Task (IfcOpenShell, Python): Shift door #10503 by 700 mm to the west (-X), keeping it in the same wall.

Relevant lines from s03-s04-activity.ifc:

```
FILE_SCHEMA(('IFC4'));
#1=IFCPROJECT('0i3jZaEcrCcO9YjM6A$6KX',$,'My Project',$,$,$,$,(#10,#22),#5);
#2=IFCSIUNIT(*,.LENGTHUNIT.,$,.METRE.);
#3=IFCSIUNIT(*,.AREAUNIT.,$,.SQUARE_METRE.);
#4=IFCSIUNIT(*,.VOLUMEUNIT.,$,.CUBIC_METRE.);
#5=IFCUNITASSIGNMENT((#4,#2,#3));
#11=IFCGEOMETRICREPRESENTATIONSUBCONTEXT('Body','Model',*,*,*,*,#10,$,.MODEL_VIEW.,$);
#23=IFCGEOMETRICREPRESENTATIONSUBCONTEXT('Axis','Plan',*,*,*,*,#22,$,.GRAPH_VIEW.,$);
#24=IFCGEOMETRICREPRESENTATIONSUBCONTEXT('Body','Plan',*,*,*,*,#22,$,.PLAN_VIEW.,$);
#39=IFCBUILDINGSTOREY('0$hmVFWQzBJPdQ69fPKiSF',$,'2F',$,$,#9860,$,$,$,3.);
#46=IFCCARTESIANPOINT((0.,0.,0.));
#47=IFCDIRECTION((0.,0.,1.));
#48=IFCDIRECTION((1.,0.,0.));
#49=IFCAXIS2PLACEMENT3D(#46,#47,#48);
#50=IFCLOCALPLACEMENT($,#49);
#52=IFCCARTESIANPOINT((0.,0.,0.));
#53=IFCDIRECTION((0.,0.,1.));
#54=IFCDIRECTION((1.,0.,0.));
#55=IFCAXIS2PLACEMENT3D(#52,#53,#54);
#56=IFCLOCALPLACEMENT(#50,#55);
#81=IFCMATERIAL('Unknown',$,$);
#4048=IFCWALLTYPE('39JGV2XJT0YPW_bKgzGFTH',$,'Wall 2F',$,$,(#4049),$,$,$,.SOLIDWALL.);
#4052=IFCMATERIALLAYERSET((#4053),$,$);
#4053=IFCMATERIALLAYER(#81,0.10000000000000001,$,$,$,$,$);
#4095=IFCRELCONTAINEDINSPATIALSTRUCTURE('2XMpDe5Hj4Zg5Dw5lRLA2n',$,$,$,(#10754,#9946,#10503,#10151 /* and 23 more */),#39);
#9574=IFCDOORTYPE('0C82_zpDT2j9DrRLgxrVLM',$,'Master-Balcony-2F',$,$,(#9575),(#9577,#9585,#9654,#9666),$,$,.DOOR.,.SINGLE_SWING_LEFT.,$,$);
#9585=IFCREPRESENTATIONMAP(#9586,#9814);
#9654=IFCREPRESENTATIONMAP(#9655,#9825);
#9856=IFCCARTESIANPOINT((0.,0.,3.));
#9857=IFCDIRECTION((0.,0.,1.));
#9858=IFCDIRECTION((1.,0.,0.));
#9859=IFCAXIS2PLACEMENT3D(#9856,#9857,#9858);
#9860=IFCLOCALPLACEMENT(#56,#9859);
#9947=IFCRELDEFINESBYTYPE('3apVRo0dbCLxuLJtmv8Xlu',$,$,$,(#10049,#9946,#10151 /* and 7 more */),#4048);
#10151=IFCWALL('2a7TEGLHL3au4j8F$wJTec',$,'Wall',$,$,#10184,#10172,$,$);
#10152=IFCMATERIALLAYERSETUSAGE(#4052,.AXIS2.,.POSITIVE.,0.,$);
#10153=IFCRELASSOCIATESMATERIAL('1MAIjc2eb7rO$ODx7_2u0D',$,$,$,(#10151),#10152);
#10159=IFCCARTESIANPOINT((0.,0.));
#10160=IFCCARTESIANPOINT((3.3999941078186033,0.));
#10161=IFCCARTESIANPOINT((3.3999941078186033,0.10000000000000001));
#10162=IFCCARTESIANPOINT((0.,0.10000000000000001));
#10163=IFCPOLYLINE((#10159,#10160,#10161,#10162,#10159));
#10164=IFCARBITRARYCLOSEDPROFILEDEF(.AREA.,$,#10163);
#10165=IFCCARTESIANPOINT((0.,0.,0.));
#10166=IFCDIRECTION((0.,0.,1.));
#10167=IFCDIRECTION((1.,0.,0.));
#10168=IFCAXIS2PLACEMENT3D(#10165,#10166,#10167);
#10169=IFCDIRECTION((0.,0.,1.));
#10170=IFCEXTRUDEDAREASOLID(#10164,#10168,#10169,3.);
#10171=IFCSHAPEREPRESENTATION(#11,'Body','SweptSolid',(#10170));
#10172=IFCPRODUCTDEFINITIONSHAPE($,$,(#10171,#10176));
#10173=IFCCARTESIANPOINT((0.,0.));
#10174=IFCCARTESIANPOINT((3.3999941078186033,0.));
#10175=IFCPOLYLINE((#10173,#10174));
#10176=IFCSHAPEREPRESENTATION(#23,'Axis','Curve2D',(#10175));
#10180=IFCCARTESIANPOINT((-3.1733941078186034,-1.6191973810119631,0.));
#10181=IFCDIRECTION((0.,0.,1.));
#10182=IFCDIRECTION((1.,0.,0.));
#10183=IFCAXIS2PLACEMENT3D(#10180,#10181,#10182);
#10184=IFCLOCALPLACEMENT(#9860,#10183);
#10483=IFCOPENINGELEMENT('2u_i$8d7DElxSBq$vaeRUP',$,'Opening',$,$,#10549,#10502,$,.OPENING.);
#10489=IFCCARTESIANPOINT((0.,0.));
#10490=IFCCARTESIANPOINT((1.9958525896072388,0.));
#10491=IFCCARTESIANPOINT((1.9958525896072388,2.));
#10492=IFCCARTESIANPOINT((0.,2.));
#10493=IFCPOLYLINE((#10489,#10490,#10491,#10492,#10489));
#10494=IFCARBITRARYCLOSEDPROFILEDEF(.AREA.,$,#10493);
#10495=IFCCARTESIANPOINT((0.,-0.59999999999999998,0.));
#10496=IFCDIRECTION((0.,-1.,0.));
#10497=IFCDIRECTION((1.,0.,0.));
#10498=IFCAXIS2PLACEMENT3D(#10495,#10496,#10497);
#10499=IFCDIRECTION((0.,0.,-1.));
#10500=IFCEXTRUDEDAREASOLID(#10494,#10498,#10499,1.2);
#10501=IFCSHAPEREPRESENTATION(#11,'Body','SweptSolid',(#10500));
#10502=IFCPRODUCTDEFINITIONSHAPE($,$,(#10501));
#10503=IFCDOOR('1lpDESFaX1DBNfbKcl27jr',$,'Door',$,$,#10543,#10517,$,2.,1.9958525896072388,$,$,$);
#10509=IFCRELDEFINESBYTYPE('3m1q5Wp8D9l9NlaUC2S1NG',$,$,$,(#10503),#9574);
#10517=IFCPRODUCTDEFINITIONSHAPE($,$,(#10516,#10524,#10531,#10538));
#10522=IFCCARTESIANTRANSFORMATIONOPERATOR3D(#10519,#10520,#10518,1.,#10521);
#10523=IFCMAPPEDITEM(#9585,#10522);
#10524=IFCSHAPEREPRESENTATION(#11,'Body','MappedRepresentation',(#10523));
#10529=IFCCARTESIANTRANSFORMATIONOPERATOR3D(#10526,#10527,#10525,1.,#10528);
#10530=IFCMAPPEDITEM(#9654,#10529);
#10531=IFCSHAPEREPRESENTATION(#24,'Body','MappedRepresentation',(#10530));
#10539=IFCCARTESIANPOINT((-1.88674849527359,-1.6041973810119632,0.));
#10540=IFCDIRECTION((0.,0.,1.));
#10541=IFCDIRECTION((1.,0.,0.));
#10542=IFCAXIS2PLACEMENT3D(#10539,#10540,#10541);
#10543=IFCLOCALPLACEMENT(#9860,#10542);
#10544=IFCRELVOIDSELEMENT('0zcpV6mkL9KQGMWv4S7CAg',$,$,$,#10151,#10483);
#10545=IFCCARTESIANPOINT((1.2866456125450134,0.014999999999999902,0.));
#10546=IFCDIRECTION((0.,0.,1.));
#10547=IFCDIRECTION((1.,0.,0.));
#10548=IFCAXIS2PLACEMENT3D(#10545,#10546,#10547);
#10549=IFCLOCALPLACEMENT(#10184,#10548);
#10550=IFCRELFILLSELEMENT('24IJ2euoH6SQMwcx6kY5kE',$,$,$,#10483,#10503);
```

```python
import ifcopenshell
import ifcopenshell.api.geometry
import ifcopenshell.util.placement

model = ifcopenshell.open("s03-s04-activity.ifc")

door = model.by_guid("1lpDESFaX1DBNfbKcl27jr")
opening = door.FillsVoids[0].RelatingOpeningElement
wall = opening.VoidsElements[0].RelatingBuildingElement

wall_matrix = ifcopenshell.util.placement.get_local_placement(wall.ObjectPlacement)
shift = wall_matrix[:3, 0] * -0.7
before = ifcopenshell.util.placement.get_local_placement(door.ObjectPlacement)[:3, 3].copy()

# The door is not placed relative to its opening, so move both.
for product in (opening, door):
    matrix = ifcopenshell.util.placement.get_local_placement(product.ObjectPlacement)
    matrix[:3, 3] += shift
    ifcopenshell.api.geometry.edit_object_placement(model, product=product, matrix=matrix, is_si=False)

after = ifcopenshell.util.placement.get_local_placement(door.ObjectPlacement)[:3, 3]
print("door moved by", (after - before).round(3) + 0.0)

model.write("s03-s04-activity_v2.ifc")
```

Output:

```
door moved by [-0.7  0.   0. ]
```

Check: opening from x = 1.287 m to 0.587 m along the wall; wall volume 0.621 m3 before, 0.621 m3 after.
